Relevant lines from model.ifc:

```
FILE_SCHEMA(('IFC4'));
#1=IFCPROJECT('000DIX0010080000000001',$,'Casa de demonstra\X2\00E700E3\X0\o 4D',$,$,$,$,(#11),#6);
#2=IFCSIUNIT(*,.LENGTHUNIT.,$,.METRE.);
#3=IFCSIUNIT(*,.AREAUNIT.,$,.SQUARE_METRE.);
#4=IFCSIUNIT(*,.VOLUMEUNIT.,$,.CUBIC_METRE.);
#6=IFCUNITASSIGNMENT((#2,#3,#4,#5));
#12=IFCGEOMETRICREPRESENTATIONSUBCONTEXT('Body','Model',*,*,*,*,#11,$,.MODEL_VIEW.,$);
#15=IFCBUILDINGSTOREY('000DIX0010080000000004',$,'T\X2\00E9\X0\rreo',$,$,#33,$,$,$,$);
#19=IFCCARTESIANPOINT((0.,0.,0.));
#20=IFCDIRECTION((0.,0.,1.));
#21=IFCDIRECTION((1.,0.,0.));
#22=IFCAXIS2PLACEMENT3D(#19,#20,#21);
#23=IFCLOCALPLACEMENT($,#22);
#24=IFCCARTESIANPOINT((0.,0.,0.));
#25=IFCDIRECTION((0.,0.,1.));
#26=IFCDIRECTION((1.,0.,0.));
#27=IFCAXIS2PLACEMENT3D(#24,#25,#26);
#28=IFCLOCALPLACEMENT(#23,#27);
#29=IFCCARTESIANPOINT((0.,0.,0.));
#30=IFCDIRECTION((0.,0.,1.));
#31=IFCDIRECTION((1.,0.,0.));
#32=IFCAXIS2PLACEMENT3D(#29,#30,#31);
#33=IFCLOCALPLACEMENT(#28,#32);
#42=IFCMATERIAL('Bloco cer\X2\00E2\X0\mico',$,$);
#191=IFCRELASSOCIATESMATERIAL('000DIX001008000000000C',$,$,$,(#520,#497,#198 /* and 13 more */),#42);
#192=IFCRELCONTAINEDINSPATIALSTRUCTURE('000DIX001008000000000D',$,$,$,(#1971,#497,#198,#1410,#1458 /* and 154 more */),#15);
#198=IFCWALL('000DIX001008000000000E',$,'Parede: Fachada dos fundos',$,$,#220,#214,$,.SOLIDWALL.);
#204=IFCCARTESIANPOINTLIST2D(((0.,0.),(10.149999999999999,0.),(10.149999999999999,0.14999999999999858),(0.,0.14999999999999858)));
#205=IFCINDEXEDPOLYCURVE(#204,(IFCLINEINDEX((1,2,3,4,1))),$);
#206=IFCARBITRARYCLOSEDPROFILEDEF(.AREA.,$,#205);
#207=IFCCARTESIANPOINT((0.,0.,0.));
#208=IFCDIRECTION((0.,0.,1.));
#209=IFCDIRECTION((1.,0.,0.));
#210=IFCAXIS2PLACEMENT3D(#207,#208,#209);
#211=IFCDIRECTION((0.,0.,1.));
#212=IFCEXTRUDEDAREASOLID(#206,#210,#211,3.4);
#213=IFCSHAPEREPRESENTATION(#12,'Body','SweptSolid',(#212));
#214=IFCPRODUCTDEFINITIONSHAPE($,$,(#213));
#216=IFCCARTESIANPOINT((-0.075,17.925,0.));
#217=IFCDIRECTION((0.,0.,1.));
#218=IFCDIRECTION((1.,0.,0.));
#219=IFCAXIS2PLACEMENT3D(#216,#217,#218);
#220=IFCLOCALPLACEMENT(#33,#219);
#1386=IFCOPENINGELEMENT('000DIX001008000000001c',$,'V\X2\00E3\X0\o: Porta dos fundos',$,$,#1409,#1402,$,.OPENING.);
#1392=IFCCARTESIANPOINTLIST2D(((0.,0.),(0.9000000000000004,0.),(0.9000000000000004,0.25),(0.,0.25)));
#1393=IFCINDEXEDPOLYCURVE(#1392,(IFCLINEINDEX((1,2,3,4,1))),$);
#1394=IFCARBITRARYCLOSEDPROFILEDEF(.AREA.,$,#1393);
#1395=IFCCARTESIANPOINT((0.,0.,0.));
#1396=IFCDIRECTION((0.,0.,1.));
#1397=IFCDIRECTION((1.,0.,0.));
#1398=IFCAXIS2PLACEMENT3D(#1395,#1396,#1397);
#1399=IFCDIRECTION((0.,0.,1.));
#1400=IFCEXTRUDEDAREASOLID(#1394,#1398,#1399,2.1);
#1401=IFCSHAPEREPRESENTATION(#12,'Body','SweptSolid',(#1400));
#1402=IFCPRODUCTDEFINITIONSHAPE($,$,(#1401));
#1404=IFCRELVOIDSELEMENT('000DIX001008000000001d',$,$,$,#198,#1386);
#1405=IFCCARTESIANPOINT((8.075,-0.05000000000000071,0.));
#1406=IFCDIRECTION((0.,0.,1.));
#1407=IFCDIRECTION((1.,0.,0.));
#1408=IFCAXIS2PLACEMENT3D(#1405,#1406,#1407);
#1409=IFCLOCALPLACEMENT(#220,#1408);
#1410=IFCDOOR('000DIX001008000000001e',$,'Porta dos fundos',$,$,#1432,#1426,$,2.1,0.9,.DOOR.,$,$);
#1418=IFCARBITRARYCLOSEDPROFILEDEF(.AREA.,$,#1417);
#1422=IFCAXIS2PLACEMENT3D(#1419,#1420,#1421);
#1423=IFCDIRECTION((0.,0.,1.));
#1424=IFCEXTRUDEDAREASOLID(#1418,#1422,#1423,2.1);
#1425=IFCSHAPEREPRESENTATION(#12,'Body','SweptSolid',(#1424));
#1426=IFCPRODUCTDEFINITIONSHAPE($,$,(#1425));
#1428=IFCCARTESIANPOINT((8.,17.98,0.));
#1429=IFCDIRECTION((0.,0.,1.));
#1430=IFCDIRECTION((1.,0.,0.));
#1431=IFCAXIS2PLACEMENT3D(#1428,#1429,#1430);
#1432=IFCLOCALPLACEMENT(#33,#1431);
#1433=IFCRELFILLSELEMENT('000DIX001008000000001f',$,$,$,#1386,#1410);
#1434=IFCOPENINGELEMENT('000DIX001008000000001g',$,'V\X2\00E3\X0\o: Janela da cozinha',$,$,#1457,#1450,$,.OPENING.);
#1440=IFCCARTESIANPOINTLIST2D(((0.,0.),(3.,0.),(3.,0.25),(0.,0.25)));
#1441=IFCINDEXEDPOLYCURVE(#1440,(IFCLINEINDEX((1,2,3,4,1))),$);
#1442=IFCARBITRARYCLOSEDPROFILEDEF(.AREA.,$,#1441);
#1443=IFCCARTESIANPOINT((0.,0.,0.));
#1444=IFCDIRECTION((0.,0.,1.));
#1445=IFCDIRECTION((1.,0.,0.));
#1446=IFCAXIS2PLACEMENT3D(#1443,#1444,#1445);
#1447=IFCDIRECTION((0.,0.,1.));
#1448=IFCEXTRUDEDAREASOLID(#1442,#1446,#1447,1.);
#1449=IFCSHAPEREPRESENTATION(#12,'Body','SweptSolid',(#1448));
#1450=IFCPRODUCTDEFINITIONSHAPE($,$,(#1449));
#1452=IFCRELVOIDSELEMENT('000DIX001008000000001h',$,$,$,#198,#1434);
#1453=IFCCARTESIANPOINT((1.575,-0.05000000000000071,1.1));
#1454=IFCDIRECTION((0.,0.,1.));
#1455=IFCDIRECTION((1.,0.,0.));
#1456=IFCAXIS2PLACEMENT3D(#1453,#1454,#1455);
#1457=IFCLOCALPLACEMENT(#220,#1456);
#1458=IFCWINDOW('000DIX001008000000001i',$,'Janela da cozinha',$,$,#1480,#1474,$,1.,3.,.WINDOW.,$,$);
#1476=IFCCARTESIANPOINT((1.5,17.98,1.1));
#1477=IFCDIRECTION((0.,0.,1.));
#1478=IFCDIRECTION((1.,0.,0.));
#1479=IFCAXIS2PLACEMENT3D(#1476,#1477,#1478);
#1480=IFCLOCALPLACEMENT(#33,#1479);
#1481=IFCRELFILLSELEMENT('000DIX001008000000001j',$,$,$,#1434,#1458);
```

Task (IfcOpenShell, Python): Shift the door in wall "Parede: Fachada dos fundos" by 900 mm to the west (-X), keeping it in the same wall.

```python
import ifcopenshell
import ifcopenshell.api.geometry
import ifcopenshell.util.placement
import ifcopenshell.util.unit

model = ifcopenshell.open("model.ifc")
unit_scale = ifcopenshell.util.unit.calculate_unit_scale(model)

door = model.by_guid("000DIX001008000000001e")
opening = door.FillsVoids[0].RelatingOpeningElement
wall = opening.VoidsElements[0].RelatingBuildingElement

wall_matrix = ifcopenshell.util.placement.get_local_placement(wall.ObjectPlacement)
shift = wall_matrix[:3, 0] * -0.9 / unit_scale
before = ifcopenshell.util.placement.get_local_placement(door.ObjectPlacement)[:3, 3].copy()

# The door is not placed relative to its opening, so move both.
for product in (opening, door):
    matrix = ifcopenshell.util.placement.get_local_placement(product.ObjectPlacement)
    matrix[:3, 3] += shift
    ifcopenshell.api.geometry.edit_object_placement(model, product=product, matrix=matrix, is_si=False)

after = ifcopenshell.util.placement.get_local_placement(door.ObjectPlacement)[:3, 3]
print("door moved by", (after - before).round(3) + 0.0)

model.write("model_updated.ifc")
```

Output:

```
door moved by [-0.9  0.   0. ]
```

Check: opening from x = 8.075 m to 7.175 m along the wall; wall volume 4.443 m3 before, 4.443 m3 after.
